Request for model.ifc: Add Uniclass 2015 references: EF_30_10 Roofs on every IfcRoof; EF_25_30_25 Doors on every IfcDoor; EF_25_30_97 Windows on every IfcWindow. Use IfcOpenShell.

First a look at what the model holds.

```python
import ifcopenshell

model = ifcopenshell.open("model.ifc")
print(model.schema)
print("classifications:", [c.Name for c in model.by_type("IfcClassification")])
for ifc_class in ("IfcDoor", "IfcRoof", "IfcStair", "IfcWall", "IfcWindow"):
    print(ifc_class, len(model.by_type(ifc_class)))
```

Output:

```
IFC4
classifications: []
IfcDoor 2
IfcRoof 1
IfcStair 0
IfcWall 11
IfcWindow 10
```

```python
import ifcopenshell
import ifcopenshell.api.classification

model = ifcopenshell.open("model.ifc")

system = ifcopenshell.api.classification.add_classification(model, classification="Uniclass 2015")

codes = {
    "IfcRoof": ("EF_30_10", "Roofs"),
    "IfcDoor": ("EF_25_30_25", "Doors"),
    "IfcWindow": ("EF_25_30_97", "Windows"),
}
for ifc_class, (code, name) in codes.items():
    products = model.by_type(ifc_class)
    ifcopenshell.api.classification.add_reference(
        model, products=products, classification=system, identification=code, name=name
    )
    print(code, len(products))

model.write("model_edited.ifc")
```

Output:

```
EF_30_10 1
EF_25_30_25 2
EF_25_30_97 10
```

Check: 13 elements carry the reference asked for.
